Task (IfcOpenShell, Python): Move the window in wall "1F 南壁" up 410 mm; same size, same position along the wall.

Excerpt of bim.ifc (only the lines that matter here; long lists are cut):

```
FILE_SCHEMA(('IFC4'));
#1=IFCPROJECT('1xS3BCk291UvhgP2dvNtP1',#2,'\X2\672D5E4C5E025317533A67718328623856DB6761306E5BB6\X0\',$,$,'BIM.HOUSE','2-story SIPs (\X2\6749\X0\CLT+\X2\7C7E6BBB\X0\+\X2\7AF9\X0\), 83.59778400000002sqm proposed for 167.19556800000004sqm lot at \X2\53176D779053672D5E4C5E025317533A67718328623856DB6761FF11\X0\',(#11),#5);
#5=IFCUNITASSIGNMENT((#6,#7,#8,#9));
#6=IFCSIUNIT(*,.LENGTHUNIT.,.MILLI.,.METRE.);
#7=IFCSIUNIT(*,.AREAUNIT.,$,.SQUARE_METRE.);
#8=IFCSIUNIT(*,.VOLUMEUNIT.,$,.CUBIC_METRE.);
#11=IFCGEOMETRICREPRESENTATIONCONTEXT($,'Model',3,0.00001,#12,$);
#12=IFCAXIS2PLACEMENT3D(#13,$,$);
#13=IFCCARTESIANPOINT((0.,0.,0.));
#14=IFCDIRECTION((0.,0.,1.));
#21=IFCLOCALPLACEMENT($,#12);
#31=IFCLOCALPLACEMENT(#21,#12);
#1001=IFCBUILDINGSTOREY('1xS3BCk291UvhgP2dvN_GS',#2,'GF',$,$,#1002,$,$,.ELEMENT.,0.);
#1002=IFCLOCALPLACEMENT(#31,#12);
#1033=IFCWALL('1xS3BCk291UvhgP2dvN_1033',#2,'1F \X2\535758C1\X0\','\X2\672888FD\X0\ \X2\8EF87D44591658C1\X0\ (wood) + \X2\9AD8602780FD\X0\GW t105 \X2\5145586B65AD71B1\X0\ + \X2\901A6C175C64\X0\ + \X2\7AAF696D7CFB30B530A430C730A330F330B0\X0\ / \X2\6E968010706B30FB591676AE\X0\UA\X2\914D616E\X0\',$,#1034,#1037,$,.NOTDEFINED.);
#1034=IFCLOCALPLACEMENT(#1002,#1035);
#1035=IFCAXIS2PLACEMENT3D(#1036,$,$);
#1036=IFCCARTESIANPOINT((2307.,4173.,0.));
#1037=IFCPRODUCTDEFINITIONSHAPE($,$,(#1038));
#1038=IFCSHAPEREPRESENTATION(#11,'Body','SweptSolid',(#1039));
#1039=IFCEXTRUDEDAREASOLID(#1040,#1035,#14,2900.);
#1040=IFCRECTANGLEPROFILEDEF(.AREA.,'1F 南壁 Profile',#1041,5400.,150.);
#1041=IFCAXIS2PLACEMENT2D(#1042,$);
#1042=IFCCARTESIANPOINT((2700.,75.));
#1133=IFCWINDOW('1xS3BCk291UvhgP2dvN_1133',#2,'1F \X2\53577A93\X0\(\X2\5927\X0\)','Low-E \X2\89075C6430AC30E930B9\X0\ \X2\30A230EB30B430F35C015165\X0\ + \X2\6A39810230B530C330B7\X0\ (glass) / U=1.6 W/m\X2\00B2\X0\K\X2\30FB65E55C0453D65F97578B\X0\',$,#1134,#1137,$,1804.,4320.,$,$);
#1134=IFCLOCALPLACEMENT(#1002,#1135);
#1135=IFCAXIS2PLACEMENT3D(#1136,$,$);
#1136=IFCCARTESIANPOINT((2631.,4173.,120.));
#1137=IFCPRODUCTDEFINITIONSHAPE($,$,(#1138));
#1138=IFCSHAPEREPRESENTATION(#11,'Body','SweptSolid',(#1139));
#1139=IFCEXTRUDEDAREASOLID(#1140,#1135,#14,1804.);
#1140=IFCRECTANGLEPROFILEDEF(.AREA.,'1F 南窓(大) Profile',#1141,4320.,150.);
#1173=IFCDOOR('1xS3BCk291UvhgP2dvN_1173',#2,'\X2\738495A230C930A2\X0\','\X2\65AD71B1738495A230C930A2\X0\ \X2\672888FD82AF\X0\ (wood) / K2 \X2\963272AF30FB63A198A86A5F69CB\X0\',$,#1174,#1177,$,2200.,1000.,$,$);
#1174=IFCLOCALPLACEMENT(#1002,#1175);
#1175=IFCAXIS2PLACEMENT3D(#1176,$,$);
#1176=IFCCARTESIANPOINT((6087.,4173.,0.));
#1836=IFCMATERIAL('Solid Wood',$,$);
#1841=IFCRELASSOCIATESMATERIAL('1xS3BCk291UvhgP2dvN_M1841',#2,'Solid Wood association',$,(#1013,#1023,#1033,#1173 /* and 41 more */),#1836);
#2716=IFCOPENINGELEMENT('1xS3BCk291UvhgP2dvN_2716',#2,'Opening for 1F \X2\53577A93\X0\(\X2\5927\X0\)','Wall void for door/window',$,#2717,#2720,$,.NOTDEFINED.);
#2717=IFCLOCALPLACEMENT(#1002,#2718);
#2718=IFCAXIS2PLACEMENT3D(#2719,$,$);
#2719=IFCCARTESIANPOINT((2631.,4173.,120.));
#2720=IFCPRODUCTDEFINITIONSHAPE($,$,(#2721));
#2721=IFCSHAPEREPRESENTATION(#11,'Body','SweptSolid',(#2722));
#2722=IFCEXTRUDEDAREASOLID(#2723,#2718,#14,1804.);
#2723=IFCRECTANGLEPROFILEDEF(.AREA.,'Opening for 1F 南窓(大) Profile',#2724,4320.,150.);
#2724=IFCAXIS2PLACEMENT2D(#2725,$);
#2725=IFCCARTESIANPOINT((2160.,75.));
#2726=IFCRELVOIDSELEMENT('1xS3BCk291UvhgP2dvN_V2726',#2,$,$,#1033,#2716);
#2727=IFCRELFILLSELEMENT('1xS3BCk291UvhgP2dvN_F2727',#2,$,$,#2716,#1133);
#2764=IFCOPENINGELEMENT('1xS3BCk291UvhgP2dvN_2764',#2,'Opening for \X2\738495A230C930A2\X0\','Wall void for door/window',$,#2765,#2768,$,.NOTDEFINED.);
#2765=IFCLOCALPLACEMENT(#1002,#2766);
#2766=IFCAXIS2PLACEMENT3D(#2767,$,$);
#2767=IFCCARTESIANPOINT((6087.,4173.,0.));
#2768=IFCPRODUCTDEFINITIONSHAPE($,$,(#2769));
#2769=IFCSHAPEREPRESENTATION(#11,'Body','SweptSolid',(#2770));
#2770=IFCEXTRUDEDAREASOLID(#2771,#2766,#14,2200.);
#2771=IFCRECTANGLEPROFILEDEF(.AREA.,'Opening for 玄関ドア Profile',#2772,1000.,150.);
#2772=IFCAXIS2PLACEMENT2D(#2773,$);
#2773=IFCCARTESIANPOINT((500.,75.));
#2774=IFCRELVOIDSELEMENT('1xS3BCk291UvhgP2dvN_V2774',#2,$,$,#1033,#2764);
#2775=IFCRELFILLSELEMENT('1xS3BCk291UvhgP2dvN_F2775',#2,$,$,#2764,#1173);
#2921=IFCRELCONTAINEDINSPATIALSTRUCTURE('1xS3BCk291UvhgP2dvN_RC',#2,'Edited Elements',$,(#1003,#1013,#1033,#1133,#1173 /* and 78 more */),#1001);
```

```python
import numpy as np
import ifcopenshell
import ifcopenshell.api.geometry
import ifcopenshell.util.placement
import ifcopenshell.util.unit

model = ifcopenshell.open("bim.ifc")
unit_scale = ifcopenshell.util.unit.calculate_unit_scale(model)

window = model.by_guid("1xS3BCk291UvhgP2dvN_1133")
opening = window.FillsVoids[0].RelatingOpeningElement
dz = 0.41 / unit_scale

shift = np.array([0.0, 0.0, dz])
# The window is not placed relative to its opening, so move both.
for product in (opening, window):
    matrix = ifcopenshell.util.placement.get_local_placement(product.ObjectPlacement)
    matrix[:3, 3] += shift
    ifcopenshell.api.geometry.edit_object_placement(model, product=product, matrix=matrix, is_si=False)

print(f"moved by {dz * unit_scale:+.3f} m")

model.write("bim_edited.ifc")
```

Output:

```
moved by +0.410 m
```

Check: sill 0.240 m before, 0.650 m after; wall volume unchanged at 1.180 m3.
